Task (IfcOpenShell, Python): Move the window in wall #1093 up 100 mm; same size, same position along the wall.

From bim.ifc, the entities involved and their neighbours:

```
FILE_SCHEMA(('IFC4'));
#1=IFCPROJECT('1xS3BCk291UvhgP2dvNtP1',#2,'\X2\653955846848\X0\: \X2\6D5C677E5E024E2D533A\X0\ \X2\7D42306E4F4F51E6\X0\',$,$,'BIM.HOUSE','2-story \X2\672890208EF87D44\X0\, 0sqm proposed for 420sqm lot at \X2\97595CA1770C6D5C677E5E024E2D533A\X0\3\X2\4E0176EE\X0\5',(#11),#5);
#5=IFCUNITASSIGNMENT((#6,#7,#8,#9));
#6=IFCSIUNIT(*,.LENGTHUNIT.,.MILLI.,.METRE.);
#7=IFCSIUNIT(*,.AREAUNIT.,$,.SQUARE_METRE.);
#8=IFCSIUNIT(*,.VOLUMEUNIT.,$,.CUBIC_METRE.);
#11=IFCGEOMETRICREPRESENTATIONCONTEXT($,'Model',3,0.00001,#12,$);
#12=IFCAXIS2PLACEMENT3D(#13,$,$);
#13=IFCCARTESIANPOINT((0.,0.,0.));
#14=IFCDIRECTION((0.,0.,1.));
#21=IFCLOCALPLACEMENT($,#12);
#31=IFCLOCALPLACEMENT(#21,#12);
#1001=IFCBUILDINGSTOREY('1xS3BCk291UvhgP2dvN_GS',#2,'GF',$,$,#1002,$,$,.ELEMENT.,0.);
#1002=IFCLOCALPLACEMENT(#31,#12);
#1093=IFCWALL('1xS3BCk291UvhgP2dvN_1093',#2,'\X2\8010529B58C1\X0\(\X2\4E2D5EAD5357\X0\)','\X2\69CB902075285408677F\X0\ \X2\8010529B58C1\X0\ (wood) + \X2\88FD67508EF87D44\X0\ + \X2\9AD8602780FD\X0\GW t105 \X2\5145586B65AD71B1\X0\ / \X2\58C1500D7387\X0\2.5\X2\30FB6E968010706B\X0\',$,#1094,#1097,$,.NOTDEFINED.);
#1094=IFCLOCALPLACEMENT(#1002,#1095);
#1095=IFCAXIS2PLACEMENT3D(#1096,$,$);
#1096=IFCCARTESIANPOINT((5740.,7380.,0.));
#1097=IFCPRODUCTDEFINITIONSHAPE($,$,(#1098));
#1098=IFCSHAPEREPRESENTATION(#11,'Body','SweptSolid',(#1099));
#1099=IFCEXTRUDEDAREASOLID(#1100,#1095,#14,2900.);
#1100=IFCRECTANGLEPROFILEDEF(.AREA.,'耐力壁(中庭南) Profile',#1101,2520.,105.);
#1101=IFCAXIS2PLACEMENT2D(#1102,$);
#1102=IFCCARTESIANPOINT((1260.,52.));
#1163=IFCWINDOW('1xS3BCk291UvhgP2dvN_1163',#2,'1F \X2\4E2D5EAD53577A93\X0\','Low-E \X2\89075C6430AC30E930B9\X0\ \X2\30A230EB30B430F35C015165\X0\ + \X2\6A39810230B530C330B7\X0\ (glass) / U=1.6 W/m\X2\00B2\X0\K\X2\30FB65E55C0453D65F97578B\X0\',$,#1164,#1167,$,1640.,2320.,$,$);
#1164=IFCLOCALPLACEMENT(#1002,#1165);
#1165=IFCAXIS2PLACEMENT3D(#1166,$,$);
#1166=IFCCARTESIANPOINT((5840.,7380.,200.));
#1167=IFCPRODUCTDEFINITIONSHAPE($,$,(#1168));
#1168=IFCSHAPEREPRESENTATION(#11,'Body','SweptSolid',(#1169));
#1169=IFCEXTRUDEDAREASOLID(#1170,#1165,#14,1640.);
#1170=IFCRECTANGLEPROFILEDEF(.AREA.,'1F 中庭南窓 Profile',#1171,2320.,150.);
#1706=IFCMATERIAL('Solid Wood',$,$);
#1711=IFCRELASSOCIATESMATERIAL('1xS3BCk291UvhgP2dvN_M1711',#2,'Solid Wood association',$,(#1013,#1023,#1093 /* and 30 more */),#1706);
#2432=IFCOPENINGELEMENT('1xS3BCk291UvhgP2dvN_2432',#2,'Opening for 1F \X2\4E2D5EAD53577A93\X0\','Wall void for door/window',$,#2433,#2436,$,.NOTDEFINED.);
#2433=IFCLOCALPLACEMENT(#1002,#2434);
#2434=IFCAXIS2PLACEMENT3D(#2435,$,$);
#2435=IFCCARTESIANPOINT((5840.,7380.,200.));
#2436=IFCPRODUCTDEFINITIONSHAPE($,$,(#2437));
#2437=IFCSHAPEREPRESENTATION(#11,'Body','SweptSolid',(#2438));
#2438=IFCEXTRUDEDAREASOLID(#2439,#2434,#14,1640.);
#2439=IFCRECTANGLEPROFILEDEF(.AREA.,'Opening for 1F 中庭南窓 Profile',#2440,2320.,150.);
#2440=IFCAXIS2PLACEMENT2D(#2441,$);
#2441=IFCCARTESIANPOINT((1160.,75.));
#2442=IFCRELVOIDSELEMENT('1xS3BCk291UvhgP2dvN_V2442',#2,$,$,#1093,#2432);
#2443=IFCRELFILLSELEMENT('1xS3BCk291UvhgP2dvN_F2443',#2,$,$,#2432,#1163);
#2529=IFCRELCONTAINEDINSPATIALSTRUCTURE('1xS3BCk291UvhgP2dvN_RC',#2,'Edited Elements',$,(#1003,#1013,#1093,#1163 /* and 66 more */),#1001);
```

```python
import numpy as np
import ifcopenshell
import ifcopenshell.api.geometry
import ifcopenshell.util.placement
import ifcopenshell.util.unit

model = ifcopenshell.open("bim.ifc")
unit_scale = ifcopenshell.util.unit.calculate_unit_scale(model)

window = model.by_guid("1xS3BCk291UvhgP2dvN_1163")
opening = window.FillsVoids[0].RelatingOpeningElement
dz = 0.1 / unit_scale

shift = np.array([0.0, 0.0, dz])
# The window is not placed relative to its opening, so move both.
for product in (opening, window):
    matrix = ifcopenshell.util.placement.get_local_placement(product.ObjectPlacement)
    matrix[:3, 3] += shift
    ifcopenshell.api.geometry.edit_object_placement(model, product=product, matrix=matrix, is_si=False)

print(f"moved by {dz * unit_scale:+.3f} m")

model.write("bim-out.ifc")
```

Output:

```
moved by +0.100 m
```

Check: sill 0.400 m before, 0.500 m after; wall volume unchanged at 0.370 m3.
